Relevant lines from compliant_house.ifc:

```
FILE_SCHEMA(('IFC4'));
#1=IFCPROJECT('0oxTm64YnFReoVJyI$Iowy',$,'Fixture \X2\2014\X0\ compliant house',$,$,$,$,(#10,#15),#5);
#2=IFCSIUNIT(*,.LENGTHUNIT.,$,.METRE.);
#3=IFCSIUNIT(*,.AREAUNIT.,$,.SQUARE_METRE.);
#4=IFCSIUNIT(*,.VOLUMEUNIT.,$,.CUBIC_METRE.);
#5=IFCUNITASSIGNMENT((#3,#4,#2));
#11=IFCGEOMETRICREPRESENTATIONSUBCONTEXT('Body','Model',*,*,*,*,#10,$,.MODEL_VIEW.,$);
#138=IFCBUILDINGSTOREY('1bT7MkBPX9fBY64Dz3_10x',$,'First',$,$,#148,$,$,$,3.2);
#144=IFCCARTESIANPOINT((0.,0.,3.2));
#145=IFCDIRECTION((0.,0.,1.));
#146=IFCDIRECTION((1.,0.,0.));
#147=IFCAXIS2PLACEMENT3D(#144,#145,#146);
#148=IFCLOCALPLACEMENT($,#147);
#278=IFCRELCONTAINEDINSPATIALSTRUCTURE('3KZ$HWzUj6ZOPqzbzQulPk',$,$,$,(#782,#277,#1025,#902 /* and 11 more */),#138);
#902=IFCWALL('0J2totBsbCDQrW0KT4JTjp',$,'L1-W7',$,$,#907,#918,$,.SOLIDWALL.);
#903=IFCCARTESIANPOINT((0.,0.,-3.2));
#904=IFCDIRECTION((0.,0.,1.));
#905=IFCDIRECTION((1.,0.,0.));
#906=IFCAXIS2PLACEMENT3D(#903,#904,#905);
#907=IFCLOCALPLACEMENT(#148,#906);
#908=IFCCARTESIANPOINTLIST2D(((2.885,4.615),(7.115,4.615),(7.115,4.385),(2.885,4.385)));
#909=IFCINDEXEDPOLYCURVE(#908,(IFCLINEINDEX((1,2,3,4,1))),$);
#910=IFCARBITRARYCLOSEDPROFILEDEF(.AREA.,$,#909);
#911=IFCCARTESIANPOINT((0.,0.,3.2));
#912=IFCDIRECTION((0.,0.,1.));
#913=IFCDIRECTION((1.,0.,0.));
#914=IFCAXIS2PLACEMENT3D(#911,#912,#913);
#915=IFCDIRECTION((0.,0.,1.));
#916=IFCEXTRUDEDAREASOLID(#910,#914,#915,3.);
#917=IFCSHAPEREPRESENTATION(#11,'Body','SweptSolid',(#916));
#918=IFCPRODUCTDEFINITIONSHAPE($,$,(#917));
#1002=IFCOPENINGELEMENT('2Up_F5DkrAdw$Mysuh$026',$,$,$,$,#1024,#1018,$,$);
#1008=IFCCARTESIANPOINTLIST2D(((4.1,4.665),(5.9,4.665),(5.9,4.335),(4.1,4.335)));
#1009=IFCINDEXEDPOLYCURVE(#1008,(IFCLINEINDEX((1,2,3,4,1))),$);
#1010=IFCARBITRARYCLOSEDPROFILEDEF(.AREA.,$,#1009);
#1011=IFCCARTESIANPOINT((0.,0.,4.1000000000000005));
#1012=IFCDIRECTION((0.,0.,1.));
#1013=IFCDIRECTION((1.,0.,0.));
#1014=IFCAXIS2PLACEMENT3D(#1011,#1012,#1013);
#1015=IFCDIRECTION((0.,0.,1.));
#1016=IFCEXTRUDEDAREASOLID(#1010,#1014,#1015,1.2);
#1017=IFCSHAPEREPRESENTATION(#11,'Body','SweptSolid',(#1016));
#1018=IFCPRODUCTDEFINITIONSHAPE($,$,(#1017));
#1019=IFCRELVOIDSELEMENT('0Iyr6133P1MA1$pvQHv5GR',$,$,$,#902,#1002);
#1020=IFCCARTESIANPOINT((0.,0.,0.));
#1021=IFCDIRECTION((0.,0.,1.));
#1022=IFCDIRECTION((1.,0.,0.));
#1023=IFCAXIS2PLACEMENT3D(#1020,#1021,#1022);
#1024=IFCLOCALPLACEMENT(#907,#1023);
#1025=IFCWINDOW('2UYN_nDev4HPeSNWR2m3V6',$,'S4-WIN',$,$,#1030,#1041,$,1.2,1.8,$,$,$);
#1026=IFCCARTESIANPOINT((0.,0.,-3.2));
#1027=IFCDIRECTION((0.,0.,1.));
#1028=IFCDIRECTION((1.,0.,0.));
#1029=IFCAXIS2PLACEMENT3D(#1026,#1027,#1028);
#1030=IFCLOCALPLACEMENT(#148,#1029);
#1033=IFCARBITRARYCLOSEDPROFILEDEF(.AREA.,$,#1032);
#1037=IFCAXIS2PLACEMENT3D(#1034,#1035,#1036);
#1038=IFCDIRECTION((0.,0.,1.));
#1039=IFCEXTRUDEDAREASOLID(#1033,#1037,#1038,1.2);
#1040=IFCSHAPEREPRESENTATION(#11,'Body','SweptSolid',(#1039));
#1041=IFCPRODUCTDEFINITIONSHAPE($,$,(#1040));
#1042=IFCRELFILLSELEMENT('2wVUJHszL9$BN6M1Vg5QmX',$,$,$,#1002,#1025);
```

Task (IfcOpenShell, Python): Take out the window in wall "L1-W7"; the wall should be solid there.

```python
import ifcopenshell
import ifcopenshell.api.feature
import ifcopenshell.api.root
import ifcopenshell.geom
import ifcopenshell.util.shape

model = ifcopenshell.open("compliant_house.ifc")
settings = ifcopenshell.geom.settings()


def volume(element):
    """Net volume in cubic metres, openings subtracted."""
    shape = ifcopenshell.geom.create_shape(settings, element)
    return ifcopenshell.util.shape.get_volume(shape.geometry)


window = model.by_guid("2UYN_nDev4HPeSNWR2m3V6")
opening = window.FillsVoids[0].RelatingOpeningElement
wall = opening.VoidsElements[0].RelatingBuildingElement
before = volume(wall)

ifcopenshell.api.root.remove_product(model, product=window)
ifcopenshell.api.feature.remove_feature(model, feature=opening)

after = volume(wall)

print(f"wall volume {before:.3f} -> {after:.3f} m3")

model.write("compliant_house_rev.ifc")
```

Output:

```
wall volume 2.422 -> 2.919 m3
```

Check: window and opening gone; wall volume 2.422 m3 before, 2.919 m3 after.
